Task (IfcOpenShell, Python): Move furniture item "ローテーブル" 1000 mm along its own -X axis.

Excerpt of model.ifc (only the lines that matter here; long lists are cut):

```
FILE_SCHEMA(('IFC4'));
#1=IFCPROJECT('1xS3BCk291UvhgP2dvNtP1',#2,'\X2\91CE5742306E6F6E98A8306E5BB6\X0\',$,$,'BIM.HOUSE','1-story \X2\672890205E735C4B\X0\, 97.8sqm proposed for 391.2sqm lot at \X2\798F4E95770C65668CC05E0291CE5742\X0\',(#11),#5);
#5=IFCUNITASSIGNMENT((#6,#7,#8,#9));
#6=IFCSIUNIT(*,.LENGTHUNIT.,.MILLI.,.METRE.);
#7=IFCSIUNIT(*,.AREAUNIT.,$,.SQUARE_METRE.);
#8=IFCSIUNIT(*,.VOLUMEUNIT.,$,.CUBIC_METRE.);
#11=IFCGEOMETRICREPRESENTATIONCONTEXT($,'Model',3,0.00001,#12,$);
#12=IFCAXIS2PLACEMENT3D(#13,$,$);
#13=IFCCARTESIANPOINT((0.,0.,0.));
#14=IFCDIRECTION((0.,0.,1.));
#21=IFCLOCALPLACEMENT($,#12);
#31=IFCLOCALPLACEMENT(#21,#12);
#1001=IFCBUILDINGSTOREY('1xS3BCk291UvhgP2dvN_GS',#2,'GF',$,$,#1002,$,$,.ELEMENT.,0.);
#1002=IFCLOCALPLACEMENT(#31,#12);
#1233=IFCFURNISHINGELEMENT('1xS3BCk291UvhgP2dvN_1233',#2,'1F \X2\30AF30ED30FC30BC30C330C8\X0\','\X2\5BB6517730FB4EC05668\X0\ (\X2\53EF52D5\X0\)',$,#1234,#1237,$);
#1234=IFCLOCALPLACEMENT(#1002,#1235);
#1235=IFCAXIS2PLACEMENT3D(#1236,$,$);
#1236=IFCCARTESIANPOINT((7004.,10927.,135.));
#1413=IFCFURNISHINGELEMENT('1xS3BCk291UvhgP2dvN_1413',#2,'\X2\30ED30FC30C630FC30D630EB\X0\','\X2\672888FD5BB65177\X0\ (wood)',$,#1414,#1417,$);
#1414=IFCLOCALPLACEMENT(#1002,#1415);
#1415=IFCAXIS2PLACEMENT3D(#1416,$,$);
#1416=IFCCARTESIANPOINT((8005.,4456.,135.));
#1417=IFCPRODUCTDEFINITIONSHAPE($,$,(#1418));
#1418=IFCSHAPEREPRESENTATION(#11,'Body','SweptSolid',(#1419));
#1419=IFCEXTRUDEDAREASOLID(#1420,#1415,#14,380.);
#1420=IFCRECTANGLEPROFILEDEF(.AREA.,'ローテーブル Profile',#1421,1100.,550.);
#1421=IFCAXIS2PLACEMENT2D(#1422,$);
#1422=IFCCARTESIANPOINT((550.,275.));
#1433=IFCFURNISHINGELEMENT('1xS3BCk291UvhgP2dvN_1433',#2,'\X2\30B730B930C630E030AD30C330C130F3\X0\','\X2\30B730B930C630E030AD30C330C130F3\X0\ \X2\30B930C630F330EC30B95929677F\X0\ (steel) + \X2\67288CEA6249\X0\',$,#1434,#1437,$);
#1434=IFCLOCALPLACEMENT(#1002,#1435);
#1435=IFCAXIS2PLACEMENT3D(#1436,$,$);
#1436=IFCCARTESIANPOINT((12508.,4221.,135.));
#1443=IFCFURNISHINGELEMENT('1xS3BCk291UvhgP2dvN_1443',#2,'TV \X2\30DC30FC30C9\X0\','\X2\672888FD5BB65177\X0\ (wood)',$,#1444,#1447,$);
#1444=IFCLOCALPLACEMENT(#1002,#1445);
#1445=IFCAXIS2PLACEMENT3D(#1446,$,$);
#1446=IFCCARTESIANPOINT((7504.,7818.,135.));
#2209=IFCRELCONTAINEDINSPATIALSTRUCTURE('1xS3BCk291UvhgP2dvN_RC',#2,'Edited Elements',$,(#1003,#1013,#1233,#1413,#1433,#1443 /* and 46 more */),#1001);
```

```python
import ifcopenshell
import ifcopenshell.api.geometry
import ifcopenshell.util.placement
import ifcopenshell.util.unit

model = ifcopenshell.open("model.ifc")
unit_scale = ifcopenshell.util.unit.calculate_unit_scale(model)

item = model.by_guid("1xS3BCk291UvhgP2dvN_1413")
matrix = ifcopenshell.util.placement.get_local_placement(item.ObjectPlacement)
matrix[:3, 3] -= matrix[:3, 0] * 1 / unit_scale
ifcopenshell.api.geometry.edit_object_placement(model, product=item, matrix=matrix, is_si=False)

print(ifcopenshell.util.placement.get_local_placement(item.ObjectPlacement).round(3) + 0.0)

model.write("model_v2.ifc")
```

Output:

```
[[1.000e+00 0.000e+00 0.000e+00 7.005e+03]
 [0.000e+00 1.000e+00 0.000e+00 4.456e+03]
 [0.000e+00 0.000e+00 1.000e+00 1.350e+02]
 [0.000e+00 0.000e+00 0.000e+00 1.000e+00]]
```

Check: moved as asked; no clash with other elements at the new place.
